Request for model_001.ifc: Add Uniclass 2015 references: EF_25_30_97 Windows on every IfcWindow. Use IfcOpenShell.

First a look at what the model holds.

```python
import ifcopenshell

model = ifcopenshell.open("model_001.ifc")
print(model.schema)
print("classifications:", [c.Name for c in model.by_type("IfcClassification")])
for ifc_class in ("IfcDoor", "IfcRoof", "IfcStair", "IfcWall", "IfcWindow"):
    print(ifc_class, len(model.by_type(ifc_class)))
```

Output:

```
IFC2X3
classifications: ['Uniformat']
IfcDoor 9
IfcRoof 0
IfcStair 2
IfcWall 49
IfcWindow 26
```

```python
import ifcopenshell
import ifcopenshell.api.classification

model = ifcopenshell.open("model_001.ifc")

# IFC2X3 requires Source and Edition and has no link from the project to the system.
system = model.create_entity("IfcClassification", Source="NBS", Edition="2015", Name="Uniclass 2015")

codes = {
    "IfcWindow": ("EF_25_30_97", "Windows"),
}
for ifc_class, (code, name) in codes.items():
    products = model.by_type(ifc_class)
    ifcopenshell.api.classification.add_reference(
        model, products=products, classification=system, identification=code, name=name
    )
    print(code, len(products))

model.write("model_001_edited.ifc")
```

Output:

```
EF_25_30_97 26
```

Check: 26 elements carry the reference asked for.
